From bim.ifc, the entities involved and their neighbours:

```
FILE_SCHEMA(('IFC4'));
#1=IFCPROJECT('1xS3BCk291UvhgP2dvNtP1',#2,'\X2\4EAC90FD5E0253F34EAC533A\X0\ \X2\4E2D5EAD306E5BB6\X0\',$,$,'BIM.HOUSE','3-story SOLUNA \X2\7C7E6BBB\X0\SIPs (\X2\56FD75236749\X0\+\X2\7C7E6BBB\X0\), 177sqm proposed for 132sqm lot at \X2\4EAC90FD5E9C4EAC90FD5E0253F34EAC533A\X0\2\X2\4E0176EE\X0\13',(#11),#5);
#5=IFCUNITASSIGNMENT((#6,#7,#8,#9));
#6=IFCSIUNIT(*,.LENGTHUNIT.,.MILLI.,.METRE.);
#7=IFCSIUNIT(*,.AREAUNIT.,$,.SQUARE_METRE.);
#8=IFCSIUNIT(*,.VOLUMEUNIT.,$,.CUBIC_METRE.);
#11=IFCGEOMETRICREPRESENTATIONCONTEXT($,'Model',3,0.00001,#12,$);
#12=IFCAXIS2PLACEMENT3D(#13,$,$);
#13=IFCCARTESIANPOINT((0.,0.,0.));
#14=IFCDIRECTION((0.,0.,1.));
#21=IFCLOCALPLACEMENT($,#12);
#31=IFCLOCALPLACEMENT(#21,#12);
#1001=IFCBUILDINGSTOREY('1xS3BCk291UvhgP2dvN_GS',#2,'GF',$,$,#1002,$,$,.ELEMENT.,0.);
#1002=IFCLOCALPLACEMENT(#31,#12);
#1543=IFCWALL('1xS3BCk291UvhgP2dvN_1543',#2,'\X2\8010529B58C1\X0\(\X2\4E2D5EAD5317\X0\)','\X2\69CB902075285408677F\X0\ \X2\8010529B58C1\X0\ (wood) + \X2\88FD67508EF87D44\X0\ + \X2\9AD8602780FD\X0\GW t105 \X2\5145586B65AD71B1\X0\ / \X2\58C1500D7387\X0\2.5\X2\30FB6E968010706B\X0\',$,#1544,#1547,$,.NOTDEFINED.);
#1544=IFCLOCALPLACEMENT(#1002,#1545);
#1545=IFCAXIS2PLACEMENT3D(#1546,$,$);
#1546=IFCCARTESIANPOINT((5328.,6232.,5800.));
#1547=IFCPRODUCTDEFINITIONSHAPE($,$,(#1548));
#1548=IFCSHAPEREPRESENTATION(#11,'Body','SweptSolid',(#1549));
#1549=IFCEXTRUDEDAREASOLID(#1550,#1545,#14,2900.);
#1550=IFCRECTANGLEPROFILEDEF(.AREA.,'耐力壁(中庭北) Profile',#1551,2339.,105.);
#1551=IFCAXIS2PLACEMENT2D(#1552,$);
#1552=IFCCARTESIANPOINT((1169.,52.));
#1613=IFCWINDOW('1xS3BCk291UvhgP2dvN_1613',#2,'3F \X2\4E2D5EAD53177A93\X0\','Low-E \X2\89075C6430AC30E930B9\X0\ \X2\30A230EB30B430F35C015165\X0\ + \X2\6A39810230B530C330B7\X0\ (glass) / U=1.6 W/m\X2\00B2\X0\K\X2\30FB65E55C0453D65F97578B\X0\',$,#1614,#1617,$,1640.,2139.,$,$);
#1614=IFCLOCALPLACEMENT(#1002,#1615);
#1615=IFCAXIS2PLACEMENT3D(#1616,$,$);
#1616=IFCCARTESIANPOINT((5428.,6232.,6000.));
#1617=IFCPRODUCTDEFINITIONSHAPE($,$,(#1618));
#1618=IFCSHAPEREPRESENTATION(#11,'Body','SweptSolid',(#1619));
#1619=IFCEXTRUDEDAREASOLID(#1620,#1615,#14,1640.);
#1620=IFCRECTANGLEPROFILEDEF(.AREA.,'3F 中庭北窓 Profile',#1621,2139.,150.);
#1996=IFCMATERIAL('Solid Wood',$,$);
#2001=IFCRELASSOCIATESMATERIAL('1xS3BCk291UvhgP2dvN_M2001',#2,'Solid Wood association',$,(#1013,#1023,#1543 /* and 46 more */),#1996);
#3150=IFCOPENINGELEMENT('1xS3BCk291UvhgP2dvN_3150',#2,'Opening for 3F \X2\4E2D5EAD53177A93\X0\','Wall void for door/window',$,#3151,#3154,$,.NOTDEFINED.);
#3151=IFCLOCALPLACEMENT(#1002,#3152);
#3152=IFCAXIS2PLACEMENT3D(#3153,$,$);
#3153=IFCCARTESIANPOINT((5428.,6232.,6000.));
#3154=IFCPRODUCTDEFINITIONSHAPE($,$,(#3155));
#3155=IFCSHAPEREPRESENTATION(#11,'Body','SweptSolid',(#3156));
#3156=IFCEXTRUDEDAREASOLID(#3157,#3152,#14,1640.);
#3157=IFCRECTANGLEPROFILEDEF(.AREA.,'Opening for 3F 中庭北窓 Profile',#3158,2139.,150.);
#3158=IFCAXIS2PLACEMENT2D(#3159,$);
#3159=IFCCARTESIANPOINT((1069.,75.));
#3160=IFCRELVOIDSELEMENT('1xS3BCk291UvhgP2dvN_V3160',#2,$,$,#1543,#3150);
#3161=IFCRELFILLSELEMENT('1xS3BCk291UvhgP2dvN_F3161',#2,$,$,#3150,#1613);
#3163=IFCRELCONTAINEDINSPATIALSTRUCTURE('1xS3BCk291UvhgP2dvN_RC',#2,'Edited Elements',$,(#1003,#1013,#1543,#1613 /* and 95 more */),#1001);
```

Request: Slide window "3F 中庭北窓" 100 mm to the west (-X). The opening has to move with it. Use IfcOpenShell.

```python
import ifcopenshell
import ifcopenshell.api.geometry
import ifcopenshell.util.placement

model = ifcopenshell.open("bim.ifc")

window = model.by_id(1613)
opening = window.FillsVoids[0].RelatingOpeningElement
wall = opening.VoidsElements[0].RelatingBuildingElement

wall_matrix = ifcopenshell.util.placement.get_local_placement(wall.ObjectPlacement)
shift = wall_matrix[:3, 0] * -100.0
before = ifcopenshell.util.placement.get_local_placement(window.ObjectPlacement)[:3, 3].copy()

# The window is not placed relative to its opening, so move both.
for product in (opening, window):
    matrix = ifcopenshell.util.placement.get_local_placement(product.ObjectPlacement)
    matrix[:3, 3] += shift
    ifcopenshell.api.geometry.edit_object_placement(model, product=product, matrix=matrix, is_si=False)

after = ifcopenshell.util.placement.get_local_placement(window.ObjectPlacement)[:3, 3]
print("window moved by", (after - before).round(3) + 0.0)

model.write("bim_rev.ifc")
```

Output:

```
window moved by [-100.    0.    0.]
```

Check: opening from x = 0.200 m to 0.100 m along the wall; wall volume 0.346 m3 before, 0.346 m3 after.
